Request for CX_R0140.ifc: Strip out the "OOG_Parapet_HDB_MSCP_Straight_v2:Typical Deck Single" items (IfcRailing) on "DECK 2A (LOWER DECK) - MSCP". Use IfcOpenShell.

First a look at what the model holds.

```python
import ifcopenshell
import ifcopenshell.util.element

model = ifcopenshell.open("CX_R0140.ifc")
print(model.schema)
storey = next(s for s in model.by_type("IfcBuildingStorey") if s.Name == "DECK 2A (LOWER DECK) - MSCP")
railings = [e for e in ifcopenshell.util.element.get_decomposition(storey) if e.is_a("IfcRailing")]
seen = {}
for e in railings:
    element_type = ifcopenshell.util.element.get_type(e)
    name = element_type.Name if element_type not in (None, e) else None
    seen[name] = seen.get(name, 0) + 1
for name, count in sorted(seen.items(), key=str):
    print(count, "x", name)
```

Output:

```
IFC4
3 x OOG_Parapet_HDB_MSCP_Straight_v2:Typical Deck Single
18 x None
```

```python
import ifcopenshell
import ifcopenshell.api.root
import ifcopenshell.util.element

model = ifcopenshell.open("CX_R0140.ifc")

storey = next(s for s in model.by_type("IfcBuildingStorey") if s.Name == "DECK 2A (LOWER DECK) - MSCP")
railings = [e for e in ifcopenshell.util.element.get_decomposition(storey) if e.is_a("IfcRailing")]
targets = [e for e in railings if (t := ifcopenshell.util.element.get_type(e)) not in (None, e) and t.Name == "OOG_Parapet_HDB_MSCP_Straight_v2:Typical Deck Single"]

for e in targets:
    ifcopenshell.api.root.remove_product(model, product=e)
print(len(targets), "removed")

model.write("CX_R0140_rev.ifc")
```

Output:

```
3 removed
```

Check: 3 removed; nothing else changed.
